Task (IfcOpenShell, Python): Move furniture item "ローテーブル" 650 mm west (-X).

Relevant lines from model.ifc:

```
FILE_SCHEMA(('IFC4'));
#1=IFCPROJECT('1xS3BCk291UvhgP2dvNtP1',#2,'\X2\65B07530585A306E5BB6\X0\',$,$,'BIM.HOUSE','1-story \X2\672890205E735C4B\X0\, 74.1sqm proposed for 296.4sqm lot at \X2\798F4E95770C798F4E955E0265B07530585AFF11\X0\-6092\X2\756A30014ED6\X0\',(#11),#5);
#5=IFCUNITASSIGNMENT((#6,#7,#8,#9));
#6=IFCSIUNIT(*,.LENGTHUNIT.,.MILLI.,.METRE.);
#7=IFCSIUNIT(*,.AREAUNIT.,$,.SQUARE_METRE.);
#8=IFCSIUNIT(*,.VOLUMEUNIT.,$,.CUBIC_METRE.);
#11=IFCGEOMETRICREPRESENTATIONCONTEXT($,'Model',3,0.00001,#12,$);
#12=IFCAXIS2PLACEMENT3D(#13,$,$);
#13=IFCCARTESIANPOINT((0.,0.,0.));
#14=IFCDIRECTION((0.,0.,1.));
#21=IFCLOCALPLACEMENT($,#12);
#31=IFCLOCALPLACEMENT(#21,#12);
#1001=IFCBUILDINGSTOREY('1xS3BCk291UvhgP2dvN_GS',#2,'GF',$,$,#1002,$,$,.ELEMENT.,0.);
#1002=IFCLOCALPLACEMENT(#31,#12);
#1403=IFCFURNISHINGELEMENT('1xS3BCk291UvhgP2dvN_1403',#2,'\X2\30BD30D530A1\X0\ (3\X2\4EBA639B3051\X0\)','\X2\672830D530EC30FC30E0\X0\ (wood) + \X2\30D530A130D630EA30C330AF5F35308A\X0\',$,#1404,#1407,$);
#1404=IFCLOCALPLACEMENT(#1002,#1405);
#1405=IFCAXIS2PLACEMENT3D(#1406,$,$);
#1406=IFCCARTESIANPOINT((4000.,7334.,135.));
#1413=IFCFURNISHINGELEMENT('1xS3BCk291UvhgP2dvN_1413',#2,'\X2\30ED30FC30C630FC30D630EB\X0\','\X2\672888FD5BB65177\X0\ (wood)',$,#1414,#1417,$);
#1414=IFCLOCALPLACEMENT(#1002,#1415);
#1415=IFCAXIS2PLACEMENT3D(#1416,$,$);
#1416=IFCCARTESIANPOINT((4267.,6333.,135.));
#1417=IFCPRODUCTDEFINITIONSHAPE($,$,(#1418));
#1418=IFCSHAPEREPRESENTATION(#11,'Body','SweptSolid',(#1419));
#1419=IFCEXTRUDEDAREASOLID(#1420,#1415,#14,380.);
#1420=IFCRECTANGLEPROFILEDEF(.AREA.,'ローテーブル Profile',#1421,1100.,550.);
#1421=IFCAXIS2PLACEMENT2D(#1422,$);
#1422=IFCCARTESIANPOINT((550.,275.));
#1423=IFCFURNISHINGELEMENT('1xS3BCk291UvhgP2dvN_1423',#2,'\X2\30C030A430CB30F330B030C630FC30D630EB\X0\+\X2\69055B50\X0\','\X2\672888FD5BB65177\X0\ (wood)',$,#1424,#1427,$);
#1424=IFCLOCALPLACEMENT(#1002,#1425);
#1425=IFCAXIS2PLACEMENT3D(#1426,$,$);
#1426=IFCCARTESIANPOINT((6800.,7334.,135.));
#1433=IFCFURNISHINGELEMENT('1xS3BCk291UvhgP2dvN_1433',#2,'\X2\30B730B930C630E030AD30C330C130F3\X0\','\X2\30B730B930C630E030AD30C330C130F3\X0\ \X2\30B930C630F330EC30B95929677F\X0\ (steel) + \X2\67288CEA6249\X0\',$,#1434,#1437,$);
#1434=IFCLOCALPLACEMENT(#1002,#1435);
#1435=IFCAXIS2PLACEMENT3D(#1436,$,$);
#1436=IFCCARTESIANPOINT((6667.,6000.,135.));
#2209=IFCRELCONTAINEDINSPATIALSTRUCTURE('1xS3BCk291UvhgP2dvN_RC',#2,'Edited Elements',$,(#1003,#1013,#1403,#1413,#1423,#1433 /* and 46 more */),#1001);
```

```python
import ifcopenshell
import ifcopenshell.api.geometry
import ifcopenshell.util.placement

model = ifcopenshell.open("model.ifc")

item = model.by_guid("1xS3BCk291UvhgP2dvN_1413")
matrix = ifcopenshell.util.placement.get_local_placement(item.ObjectPlacement)
matrix[0, 3] -= 650.0
ifcopenshell.api.geometry.edit_object_placement(model, product=item, matrix=matrix, is_si=False)

print(ifcopenshell.util.placement.get_local_placement(item.ObjectPlacement).round(3) + 0.0)

model.write("model_updated.ifc")
```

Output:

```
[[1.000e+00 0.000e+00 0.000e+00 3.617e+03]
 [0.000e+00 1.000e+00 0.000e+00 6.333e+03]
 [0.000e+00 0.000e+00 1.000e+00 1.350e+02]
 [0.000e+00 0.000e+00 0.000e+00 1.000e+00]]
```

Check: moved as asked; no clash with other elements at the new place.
